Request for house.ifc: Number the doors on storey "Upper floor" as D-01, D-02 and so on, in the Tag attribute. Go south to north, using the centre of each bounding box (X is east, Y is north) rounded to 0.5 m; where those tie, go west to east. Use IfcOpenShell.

First a look at what the model holds.

```python
import ifcopenshell
import ifcopenshell.util.element
import ifcopenshell.util.placement

model = ifcopenshell.open("house.ifc")
print(model.schema)
storey = next(s for s in model.by_type("IfcBuildingStorey") if s.Name == "Upper floor")
doors = [e for e in ifcopenshell.util.element.get_decomposition(storey) if e.is_a("IfcDoor")]
for e in sorted(doors, key=lambda e: e.id()):
    origin = ifcopenshell.util.placement.get_local_placement(e.ObjectPlacement)[:3, 3]
    print(e.id(), e.Tag, e.Name, origin.round(2) + 0.0, sep=" | ")
```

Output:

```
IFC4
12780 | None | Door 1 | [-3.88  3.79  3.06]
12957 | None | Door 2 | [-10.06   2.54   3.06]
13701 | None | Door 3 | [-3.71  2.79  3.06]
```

```python
import ifcopenshell
import ifcopenshell.geom
import ifcopenshell.util.element
import ifcopenshell.util.shape

model = ifcopenshell.open("house.ifc")
settings = ifcopenshell.geom.settings()
settings.set("use-world-coords", True)


def centre(element):
    shape = ifcopenshell.geom.create_shape(settings, element)
    return ifcopenshell.util.shape.get_bbox_centroid(shape.geometry)


storey = next(s for s in model.by_type("IfcBuildingStorey") if s.Name == "Upper floor")
doors = [e for e in ifcopenshell.util.element.get_decomposition(storey) if e.is_a("IfcDoor")]

# Insertion points can sit at a corner or the storey origin, so sort by the geometry (in metres).
centres = {e: centre(e) for e in doors}
doors.sort(key=lambda e: (round(centres[e][1] / 0.5), centres[e][0]))

for i, e in enumerate(doors, start=1):
    number = f"D-{i:02d}"
    e.Tag = number
    print(e.id(), number)

model.write("house_rev.ifc")
```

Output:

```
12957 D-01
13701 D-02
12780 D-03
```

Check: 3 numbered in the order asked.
